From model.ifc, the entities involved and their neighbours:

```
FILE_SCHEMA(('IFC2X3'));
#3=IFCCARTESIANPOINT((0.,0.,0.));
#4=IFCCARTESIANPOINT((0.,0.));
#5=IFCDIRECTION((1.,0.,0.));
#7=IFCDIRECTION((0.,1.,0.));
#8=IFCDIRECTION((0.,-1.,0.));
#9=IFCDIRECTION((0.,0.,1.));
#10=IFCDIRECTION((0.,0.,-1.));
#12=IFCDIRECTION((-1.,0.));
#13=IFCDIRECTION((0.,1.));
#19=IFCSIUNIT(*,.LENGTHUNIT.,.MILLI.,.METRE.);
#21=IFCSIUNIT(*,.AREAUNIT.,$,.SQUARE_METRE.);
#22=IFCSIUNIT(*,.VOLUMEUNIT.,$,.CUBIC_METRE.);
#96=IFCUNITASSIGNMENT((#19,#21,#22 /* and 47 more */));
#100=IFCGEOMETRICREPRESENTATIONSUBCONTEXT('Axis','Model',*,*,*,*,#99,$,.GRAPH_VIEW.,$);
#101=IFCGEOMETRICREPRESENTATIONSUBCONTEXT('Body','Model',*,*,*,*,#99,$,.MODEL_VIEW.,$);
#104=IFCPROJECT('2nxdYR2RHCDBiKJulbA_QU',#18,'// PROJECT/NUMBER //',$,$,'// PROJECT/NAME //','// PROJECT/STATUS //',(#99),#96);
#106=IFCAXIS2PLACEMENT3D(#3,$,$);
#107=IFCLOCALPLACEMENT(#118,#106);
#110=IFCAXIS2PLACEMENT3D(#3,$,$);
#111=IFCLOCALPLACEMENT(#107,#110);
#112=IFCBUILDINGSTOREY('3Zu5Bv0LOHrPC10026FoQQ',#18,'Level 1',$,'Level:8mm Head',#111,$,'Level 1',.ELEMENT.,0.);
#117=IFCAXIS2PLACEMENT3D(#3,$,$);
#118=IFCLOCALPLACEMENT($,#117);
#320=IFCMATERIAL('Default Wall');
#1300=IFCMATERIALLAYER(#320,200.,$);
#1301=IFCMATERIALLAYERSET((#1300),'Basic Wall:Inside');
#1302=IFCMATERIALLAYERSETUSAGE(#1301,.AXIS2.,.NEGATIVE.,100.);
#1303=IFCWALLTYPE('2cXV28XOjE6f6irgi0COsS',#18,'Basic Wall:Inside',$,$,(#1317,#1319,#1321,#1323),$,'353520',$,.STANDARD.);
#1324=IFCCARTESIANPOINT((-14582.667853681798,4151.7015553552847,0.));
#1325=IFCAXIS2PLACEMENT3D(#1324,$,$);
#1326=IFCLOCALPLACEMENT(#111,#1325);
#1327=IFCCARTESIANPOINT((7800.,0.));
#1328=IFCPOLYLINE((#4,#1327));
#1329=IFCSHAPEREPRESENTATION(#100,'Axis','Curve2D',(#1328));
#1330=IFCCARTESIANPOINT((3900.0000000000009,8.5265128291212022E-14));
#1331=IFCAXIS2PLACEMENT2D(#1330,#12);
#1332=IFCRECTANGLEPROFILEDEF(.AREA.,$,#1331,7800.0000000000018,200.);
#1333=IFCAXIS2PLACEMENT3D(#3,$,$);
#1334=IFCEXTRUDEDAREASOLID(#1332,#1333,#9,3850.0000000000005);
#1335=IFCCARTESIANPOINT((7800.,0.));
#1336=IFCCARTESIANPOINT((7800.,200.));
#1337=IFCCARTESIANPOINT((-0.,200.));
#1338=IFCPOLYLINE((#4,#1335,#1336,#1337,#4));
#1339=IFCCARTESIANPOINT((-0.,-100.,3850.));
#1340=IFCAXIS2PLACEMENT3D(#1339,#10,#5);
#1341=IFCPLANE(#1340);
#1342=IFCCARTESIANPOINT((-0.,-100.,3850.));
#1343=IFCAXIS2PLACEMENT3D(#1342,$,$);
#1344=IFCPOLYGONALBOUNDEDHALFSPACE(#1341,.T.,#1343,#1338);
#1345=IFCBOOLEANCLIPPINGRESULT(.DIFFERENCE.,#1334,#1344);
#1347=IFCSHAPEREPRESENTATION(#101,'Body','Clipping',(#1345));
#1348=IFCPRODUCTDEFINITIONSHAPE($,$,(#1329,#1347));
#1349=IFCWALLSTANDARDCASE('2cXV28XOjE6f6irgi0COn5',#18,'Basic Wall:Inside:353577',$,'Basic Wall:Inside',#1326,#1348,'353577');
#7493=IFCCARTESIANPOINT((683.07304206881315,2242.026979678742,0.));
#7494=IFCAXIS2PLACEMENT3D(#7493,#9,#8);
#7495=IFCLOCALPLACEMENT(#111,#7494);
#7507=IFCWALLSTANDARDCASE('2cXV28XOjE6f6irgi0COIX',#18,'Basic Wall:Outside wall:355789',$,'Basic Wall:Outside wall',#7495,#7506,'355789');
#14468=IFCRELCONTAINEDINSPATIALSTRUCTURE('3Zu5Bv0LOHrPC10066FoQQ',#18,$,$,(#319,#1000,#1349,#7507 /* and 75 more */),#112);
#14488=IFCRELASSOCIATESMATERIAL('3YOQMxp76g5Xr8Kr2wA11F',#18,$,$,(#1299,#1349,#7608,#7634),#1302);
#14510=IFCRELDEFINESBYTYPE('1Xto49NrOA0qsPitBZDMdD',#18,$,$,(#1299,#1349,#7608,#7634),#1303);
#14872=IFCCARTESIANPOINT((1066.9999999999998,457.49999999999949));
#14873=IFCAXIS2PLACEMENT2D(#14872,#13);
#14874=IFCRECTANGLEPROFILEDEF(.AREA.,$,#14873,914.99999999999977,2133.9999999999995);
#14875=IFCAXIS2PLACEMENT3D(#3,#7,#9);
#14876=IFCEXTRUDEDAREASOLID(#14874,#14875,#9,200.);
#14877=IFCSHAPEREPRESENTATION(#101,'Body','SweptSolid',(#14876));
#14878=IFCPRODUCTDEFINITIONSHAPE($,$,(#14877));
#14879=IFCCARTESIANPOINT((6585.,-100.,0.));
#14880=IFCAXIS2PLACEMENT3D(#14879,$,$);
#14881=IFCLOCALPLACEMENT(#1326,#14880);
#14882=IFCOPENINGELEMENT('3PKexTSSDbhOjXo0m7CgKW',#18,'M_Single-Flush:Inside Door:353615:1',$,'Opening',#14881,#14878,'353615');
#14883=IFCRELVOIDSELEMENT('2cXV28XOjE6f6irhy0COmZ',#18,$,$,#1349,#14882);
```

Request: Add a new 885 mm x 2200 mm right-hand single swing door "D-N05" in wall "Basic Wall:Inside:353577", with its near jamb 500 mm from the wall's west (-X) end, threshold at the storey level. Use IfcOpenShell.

```python
import numpy as np
import ifcopenshell
import ifcopenshell.api.feature
import ifcopenshell.api.geometry
import ifcopenshell.api.root
import ifcopenshell.api.spatial
import ifcopenshell.api.type
import ifcopenshell.geom
import ifcopenshell.util.element
import ifcopenshell.util.placement
import ifcopenshell.util.representation
import ifcopenshell.util.shape
import ifcopenshell.util.unit

model = ifcopenshell.open("model.ifc")
unit_scale = ifcopenshell.util.unit.calculate_unit_scale(model)
settings = ifcopenshell.geom.settings()


def volume(element):
    """Net volume in cubic metres, openings subtracted."""
    shape = ifcopenshell.geom.create_shape(settings, element)
    return ifcopenshell.util.shape.get_volume(shape.geometry)


wall = model.by_guid("2cXV28XOjE6f6irgi0COn5")
storey = ifcopenshell.util.element.get_container(wall, ifc_class="IfcBuildingStorey")
context = ifcopenshell.util.representation.get_context(model, "Model", "Body", "MODEL_VIEW")
before = volume(wall)

width, height, from_end, sill = 0.885, 2.2, 0.5, 0.0  # metres

# The wall runs along its own X axis, and the end named is its -X end.
wall_shape = ifcopenshell.geom.create_shape(settings, wall)
x, y, z = ifcopenshell.util.shape.get_vertices(wall_shape.geometry).T
start = x.min() + from_end
face, thickness = float(y.min()), float(y.max() - y.min())
wall_matrix = ifcopenshell.util.placement.get_local_placement(wall.ObjectPlacement)
level = ifcopenshell.util.placement.get_local_placement(storey.ObjectPlacement)[2, 3]


def in_wall(x, y):
    """Placement at x, y metres in the wall's axes, at sill height."""
    matrix = wall_matrix.copy()
    matrix[:, 3] = wall_matrix @ np.array([x / unit_scale, y / unit_scale, 0.0, 1.0])
    matrix[2, 3] = level + sill / unit_scale
    return matrix


# Opening: a box that overshoots both wall faces by 50 mm.
opening = ifcopenshell.api.root.create_entity(model, ifc_class="IfcOpeningElement")
box = ifcopenshell.api.geometry.add_wall_representation(
    model, context=context, length=width, height=height, thickness=thickness + 0.1
)
ifcopenshell.api.geometry.assign_representation(model, product=opening, representation=box)
ifcopenshell.api.geometry.edit_object_placement(model, product=opening, matrix=in_wall(start, face - 0.05), is_si=False)
ifcopenshell.api.feature.add_feature(model, feature=opening, element=wall)

door = ifcopenshell.api.root.create_entity(model, ifc_class="IfcDoor", name="D-N05")
door.OverallWidth, door.OverallHeight = width / unit_scale, height / unit_scale
body = ifcopenshell.api.geometry.add_door_representation(
    model,
    context=context,
    overall_width=door.OverallWidth,
    overall_height=door.OverallHeight,
    operation_type="SINGLE_SWING_RIGHT",
    lining_properties={"LiningDepth": thickness / unit_scale, "ThresholdDepth": thickness / unit_scale},
)
ifcopenshell.api.geometry.assign_representation(model, product=door, representation=body)
ifcopenshell.api.spatial.assign_container(model, products=[door], relating_structure=storey)
fills = ifcopenshell.api.feature.add_filling(model, opening=opening, element=door)
fills.OwnerHistory = door.OwnerHistory  # required in IFC2X3

# IFC2X3 keeps the operation on the door style.
style = ifcopenshell.api.root.create_entity(model, ifc_class="IfcDoorStyle", name="D-N05")
style.OperationType, style.ConstructionType = "SINGLE_SWING_RIGHT", "NOTDEFINED"
style.ParameterTakesPrecedence = style.Sizeable = False
ifcopenshell.api.type.assign_type(model, related_objects=[door], relating_type=style)

# The lining spans the wall, so the door starts at the wall face.
ifcopenshell.api.geometry.edit_object_placement(model, product=door, matrix=in_wall(start, face), is_si=False)

after = volume(wall)

print(f"wall volume {before:.3f} -> {after:.3f} m3")

model.write("model_v2.ifc")
```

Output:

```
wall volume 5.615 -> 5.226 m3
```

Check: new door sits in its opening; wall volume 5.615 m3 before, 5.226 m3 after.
